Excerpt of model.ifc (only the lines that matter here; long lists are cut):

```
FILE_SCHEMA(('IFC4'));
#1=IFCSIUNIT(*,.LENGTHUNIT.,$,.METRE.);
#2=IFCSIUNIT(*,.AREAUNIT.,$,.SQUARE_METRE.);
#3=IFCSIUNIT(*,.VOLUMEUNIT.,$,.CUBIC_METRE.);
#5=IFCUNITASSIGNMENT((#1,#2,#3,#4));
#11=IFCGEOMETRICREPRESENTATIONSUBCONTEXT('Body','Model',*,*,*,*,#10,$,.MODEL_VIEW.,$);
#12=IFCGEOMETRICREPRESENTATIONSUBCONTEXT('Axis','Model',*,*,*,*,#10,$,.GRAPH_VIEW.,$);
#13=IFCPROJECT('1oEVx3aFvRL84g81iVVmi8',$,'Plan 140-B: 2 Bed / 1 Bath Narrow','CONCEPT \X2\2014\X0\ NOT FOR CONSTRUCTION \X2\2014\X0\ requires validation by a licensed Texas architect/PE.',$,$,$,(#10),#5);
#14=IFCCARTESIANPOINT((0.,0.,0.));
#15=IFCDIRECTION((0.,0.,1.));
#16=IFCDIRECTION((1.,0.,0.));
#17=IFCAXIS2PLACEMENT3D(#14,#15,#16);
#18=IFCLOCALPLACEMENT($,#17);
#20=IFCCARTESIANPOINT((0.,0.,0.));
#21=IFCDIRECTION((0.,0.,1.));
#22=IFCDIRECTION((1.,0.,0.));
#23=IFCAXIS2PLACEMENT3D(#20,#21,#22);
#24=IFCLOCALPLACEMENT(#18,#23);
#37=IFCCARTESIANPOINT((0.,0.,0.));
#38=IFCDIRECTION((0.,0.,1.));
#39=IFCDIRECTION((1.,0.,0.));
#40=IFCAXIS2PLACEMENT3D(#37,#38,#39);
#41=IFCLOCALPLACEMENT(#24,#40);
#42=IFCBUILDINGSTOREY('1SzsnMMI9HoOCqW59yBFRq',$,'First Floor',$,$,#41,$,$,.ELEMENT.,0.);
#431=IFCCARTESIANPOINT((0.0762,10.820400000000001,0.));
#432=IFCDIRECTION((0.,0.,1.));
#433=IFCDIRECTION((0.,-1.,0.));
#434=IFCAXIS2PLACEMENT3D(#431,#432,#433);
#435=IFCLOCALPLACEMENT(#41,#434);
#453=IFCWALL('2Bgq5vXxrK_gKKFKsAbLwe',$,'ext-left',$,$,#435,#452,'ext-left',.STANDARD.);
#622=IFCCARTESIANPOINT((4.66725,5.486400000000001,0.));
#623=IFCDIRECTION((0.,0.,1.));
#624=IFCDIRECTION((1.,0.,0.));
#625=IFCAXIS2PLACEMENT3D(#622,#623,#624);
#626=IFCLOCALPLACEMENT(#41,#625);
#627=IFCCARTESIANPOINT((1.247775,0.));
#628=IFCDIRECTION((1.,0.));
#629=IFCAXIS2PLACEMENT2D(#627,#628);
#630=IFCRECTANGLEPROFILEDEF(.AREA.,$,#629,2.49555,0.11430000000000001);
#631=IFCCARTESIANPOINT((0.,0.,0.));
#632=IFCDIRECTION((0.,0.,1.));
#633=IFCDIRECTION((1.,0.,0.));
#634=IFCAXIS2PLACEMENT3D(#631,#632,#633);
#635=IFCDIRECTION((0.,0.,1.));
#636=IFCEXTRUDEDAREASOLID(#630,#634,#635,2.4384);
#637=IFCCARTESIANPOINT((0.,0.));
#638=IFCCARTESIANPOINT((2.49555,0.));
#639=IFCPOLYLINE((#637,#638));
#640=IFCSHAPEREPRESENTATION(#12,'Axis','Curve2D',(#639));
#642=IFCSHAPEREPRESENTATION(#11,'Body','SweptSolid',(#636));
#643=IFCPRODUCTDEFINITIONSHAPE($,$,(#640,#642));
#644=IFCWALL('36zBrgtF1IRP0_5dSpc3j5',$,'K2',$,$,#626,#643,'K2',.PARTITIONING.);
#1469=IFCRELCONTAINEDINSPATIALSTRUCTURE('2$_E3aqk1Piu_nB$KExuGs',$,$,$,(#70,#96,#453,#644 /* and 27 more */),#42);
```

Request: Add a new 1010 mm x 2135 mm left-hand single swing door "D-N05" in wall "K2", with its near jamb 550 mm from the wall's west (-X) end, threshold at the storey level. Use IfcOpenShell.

```python
import numpy as np
import ifcopenshell
import ifcopenshell.api.feature
import ifcopenshell.api.geometry
import ifcopenshell.api.root
import ifcopenshell.api.spatial
import ifcopenshell.geom
import ifcopenshell.util.element
import ifcopenshell.util.placement
import ifcopenshell.util.representation
import ifcopenshell.util.shape
import ifcopenshell.util.unit

model = ifcopenshell.open("model.ifc")
unit_scale = ifcopenshell.util.unit.calculate_unit_scale(model)
settings = ifcopenshell.geom.settings()


def volume(element):
    """Net volume in cubic metres, openings subtracted."""
    shape = ifcopenshell.geom.create_shape(settings, element)
    return ifcopenshell.util.shape.get_volume(shape.geometry)


wall = model.by_guid("36zBrgtF1IRP0_5dSpc3j5")
storey = ifcopenshell.util.element.get_container(wall, ifc_class="IfcBuildingStorey")
context = ifcopenshell.util.representation.get_context(model, "Model", "Body", "MODEL_VIEW")
before = volume(wall)

width, height, from_end, sill = 1.01, 2.135, 0.55, 0.0  # metres

# The wall runs along its own X axis, and the end named is its -X end.
wall_shape = ifcopenshell.geom.create_shape(settings, wall)
x, y, z = ifcopenshell.util.shape.get_vertices(wall_shape.geometry).T
start = x.min() + from_end
face, thickness = float(y.min()), float(y.max() - y.min())
wall_matrix = ifcopenshell.util.placement.get_local_placement(wall.ObjectPlacement)
level = ifcopenshell.util.placement.get_local_placement(storey.ObjectPlacement)[2, 3]


def in_wall(x, y):
    """Placement at x, y metres in the wall's axes, at sill height."""
    matrix = wall_matrix.copy()
    matrix[:, 3] = wall_matrix @ np.array([x / unit_scale, y / unit_scale, 0.0, 1.0])
    matrix[2, 3] = level + sill / unit_scale
    return matrix


# Opening: a box that overshoots both wall faces by 50 mm.
opening = ifcopenshell.api.root.create_entity(model, ifc_class="IfcOpeningElement", predefined_type="OPENING")
box = ifcopenshell.api.geometry.add_wall_representation(
    model, context=context, length=width, height=height, thickness=thickness + 0.1
)
ifcopenshell.api.geometry.assign_representation(model, product=opening, representation=box)
ifcopenshell.api.geometry.edit_object_placement(model, product=opening, matrix=in_wall(start, face - 0.05), is_si=False)
ifcopenshell.api.feature.add_feature(model, feature=opening, element=wall)

door = ifcopenshell.api.root.create_entity(model, ifc_class="IfcDoor", name="D-N05", predefined_type="DOOR")
door.OverallWidth, door.OverallHeight = width / unit_scale, height / unit_scale
door.OperationType = "SINGLE_SWING_LEFT"
body = ifcopenshell.api.geometry.add_door_representation(
    model,
    context=context,
    overall_width=door.OverallWidth,
    overall_height=door.OverallHeight,
    operation_type="SINGLE_SWING_LEFT",
    lining_properties={"LiningDepth": thickness / unit_scale, "ThresholdDepth": thickness / unit_scale},
)
ifcopenshell.api.geometry.assign_representation(model, product=door, representation=body)
ifcopenshell.api.spatial.assign_container(model, products=[door], relating_structure=storey)
ifcopenshell.api.feature.add_filling(model, opening=opening, element=door)

# The lining spans the wall, so the door starts at the wall face.
ifcopenshell.api.geometry.edit_object_placement(model, product=door, matrix=in_wall(start, face), is_si=False)

after = volume(wall)

print(f"wall volume {before:.3f} -> {after:.3f} m3")

model.write("model_edited.ifc")
```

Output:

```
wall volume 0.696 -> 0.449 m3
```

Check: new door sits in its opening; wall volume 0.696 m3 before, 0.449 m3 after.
